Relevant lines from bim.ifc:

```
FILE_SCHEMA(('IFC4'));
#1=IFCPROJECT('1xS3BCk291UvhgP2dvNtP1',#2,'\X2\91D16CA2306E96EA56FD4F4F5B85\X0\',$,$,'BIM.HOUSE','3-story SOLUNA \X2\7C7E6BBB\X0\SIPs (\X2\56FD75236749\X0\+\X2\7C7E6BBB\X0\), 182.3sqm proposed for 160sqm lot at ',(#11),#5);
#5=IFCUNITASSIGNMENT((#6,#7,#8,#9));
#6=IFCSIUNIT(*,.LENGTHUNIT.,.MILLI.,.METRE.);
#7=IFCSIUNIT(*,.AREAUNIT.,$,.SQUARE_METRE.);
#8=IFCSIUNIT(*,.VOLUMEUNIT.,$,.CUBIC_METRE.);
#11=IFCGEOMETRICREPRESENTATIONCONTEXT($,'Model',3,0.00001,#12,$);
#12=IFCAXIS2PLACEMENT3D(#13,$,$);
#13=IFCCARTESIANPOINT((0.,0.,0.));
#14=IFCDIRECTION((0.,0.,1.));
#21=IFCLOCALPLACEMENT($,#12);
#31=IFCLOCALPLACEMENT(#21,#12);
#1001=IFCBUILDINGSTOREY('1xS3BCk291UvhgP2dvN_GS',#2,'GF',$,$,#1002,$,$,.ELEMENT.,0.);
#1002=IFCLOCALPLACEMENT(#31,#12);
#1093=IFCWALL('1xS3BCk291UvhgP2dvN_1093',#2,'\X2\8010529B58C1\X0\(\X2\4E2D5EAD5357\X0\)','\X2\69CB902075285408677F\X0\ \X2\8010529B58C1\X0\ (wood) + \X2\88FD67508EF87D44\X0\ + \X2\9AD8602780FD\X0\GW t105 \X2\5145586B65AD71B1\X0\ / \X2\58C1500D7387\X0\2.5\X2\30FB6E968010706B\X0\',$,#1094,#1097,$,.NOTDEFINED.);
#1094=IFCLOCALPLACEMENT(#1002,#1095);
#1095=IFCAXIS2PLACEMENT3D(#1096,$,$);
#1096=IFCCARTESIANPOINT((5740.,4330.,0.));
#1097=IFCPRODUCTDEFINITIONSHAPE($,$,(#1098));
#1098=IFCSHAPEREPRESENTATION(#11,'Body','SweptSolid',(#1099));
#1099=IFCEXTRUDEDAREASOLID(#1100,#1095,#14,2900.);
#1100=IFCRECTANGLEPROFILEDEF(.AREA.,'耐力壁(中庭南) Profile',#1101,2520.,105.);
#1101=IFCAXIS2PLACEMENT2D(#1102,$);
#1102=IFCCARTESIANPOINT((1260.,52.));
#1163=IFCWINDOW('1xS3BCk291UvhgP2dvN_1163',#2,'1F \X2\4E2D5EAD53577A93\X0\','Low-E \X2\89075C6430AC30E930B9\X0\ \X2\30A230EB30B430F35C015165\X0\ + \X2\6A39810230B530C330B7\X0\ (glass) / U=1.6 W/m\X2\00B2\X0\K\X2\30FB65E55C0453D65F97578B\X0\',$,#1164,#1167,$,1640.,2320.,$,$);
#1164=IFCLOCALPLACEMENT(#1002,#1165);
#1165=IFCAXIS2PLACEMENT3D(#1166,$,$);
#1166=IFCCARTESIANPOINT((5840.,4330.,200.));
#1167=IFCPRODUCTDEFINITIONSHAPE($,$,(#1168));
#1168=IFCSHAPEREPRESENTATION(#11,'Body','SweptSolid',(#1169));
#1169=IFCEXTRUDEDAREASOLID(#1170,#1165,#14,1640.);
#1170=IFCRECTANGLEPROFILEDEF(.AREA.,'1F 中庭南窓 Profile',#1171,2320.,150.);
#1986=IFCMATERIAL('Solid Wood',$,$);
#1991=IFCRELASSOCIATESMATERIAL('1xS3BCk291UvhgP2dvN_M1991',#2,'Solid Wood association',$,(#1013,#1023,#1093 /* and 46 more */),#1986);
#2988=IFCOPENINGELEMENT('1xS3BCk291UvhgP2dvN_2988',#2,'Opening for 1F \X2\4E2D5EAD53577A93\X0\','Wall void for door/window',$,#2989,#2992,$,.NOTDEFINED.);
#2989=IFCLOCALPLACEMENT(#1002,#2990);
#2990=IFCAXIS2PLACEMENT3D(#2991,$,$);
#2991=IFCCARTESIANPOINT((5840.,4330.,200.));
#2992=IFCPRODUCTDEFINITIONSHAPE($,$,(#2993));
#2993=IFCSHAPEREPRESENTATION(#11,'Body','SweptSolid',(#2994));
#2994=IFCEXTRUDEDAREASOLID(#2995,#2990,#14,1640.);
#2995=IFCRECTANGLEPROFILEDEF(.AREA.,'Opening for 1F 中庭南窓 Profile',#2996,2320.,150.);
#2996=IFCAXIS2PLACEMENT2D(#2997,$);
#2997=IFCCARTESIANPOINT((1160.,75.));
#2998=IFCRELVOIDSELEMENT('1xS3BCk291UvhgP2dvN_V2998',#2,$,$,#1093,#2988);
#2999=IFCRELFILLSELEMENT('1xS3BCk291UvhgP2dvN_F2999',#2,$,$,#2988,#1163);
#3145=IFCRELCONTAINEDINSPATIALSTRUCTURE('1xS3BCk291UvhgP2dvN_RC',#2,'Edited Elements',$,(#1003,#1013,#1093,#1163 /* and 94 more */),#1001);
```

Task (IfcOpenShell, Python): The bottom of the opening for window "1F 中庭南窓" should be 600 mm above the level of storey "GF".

```python
import numpy as np
import ifcopenshell
import ifcopenshell.api.geometry
import ifcopenshell.geom
import ifcopenshell.util.element
import ifcopenshell.util.placement
import ifcopenshell.util.shape
import ifcopenshell.util.unit

model = ifcopenshell.open("bim.ifc")
unit_scale = ifcopenshell.util.unit.calculate_unit_scale(model)

window = model.by_guid("1xS3BCk291UvhgP2dvN_1163")
opening = window.FillsVoids[0].RelatingOpeningElement
storey = ifcopenshell.util.element.get_container(window, ifc_class="IfcBuildingStorey")
level = ifcopenshell.util.placement.get_local_placement(storey.ObjectPlacement)[2, 3]

# The opening's origin need not be at the sill, so measure its lowest point.
shape = ifcopenshell.geom.create_shape(ifcopenshell.geom.settings(), opening)
bottom = ifcopenshell.util.shape.get_shape_bottom_elevation(shape, shape.geometry) / unit_scale
dz = level + 0.6 / unit_scale - bottom

shift = np.array([0.0, 0.0, dz])
# The window is not placed relative to its opening, so move both.
for product in (opening, window):
    matrix = ifcopenshell.util.placement.get_local_placement(product.ObjectPlacement)
    matrix[:3, 3] += shift
    ifcopenshell.api.geometry.edit_object_placement(model, product=product, matrix=matrix, is_si=False)

print(f"moved by {dz * unit_scale:+.3f} m")

model.write("bim-out.ifc")
```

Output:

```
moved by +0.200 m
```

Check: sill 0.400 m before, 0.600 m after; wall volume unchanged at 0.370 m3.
